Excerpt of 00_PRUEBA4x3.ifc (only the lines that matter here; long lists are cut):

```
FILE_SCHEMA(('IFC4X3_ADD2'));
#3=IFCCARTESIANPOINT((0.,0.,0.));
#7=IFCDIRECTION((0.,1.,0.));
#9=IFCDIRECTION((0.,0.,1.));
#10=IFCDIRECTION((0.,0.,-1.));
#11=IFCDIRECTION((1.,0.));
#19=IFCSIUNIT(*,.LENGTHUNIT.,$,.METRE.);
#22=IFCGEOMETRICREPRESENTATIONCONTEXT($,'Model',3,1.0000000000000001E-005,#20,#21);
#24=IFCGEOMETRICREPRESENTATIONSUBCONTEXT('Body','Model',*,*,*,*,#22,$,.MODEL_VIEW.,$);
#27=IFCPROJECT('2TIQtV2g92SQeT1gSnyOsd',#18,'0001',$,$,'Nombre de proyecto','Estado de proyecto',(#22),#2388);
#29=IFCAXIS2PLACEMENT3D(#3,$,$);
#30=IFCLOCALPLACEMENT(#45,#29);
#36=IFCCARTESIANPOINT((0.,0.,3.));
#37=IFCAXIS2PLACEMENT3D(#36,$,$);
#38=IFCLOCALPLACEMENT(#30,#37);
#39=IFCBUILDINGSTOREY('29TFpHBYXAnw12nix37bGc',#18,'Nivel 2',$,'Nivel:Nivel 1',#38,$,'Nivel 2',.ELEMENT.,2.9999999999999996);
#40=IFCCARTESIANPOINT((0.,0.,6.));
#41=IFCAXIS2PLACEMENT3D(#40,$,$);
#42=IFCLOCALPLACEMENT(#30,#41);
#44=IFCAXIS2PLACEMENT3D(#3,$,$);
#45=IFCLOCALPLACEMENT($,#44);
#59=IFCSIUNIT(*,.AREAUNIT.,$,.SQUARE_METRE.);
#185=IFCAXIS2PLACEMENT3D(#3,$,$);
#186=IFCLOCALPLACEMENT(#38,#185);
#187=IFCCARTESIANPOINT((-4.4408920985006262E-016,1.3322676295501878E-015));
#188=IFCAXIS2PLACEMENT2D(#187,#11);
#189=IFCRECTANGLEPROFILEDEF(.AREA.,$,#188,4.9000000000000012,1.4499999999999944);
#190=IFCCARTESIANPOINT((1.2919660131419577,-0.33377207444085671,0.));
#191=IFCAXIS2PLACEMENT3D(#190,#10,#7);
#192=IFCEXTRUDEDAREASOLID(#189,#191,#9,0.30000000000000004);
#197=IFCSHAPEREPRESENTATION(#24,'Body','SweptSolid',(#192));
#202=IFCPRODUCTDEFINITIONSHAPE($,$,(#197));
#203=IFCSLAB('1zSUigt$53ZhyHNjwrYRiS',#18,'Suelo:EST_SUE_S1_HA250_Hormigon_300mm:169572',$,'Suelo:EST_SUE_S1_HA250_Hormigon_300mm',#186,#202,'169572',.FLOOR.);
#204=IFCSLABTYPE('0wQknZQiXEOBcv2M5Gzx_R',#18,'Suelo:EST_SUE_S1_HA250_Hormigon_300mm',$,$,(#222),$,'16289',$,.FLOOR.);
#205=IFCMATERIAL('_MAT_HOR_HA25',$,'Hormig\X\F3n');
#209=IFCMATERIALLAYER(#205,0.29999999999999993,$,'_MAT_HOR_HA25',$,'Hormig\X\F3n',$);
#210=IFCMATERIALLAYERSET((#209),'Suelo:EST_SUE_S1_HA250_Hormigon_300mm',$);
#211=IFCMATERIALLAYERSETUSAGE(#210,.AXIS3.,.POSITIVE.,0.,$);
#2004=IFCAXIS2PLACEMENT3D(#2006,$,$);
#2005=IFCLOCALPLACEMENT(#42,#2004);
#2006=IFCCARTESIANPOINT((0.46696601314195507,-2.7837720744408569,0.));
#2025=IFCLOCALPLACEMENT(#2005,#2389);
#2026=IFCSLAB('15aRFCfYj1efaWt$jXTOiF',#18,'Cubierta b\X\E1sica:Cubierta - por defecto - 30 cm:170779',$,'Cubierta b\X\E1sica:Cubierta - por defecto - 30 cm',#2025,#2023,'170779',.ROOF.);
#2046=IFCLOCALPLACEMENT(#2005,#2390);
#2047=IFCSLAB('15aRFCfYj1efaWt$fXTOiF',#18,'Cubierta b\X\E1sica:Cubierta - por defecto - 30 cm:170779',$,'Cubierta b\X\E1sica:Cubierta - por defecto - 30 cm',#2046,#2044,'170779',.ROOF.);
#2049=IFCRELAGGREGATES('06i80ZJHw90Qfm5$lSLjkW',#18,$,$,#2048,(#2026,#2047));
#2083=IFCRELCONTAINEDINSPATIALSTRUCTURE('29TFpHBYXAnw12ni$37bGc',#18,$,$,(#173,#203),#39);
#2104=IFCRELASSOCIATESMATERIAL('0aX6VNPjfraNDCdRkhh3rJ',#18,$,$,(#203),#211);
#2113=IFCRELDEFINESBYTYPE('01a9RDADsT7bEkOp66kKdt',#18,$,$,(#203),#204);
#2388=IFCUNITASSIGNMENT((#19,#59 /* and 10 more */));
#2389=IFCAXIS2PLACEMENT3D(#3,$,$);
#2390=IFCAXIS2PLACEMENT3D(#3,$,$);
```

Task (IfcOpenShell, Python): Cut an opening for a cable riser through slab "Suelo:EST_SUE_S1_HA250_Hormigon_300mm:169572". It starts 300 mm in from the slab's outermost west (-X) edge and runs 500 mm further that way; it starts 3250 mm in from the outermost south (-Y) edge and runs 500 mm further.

```python
import numpy as np
import ifcopenshell
import ifcopenshell.api.feature
import ifcopenshell.api.geometry
import ifcopenshell.api.root
import ifcopenshell.geom
import ifcopenshell.util.placement
import ifcopenshell.util.representation
import ifcopenshell.util.shape
import ifcopenshell.util.unit

model = ifcopenshell.open("00_PRUEBA4x3.ifc")
unit_scale = ifcopenshell.util.unit.calculate_unit_scale(model)
settings = ifcopenshell.geom.settings()


def volume(element):
    """Net volume in cubic metres, openings subtracted."""
    shape = ifcopenshell.geom.create_shape(settings, element)
    return ifcopenshell.util.shape.get_volume(shape.geometry)


slab = model.by_guid("1zSUigt$53ZhyHNjwrYRiS")
before = volume(slab)

# Extent in the slab's own axes, in metres. The edges named are its -X and -Y sides.
slab_shape = ifcopenshell.geom.create_shape(settings, slab)
vertices = ifcopenshell.util.shape.get_vertices(slab_shape.geometry)
x_min, y_min, bottom = vertices.min(axis=0)
top = vertices[:, 2].max()

opening = ifcopenshell.api.root.create_entity(model, ifc_class="IfcOpeningElement", name="Cable riser opening", predefined_type="OPENING")
context = ifcopenshell.util.representation.get_context(model, "Model", "Body", "MODEL_VIEW")
width, depth = 0.5, 0.5
outline = [(0.0, 0.0), (width, 0.0), (width, depth), (0.0, depth), (0.0, 0.0)]
# Overshoot both faces by 50 mm so the cut is clean.
shape = ifcopenshell.api.geometry.add_slab_representation(
    model, context=context, depth=top - bottom + 0.1, polyline=outline
)
ifcopenshell.api.geometry.assign_representation(model, product=opening, representation=shape)

matrix = ifcopenshell.util.placement.get_local_placement(slab.ObjectPlacement)
matrix[:, 3] = matrix @ np.append(np.array([x_min + 0.3, y_min + 3.25, bottom - 0.05]) / unit_scale, 1.0)
ifcopenshell.api.geometry.edit_object_placement(model, product=opening, matrix=matrix, is_si=False)
ifcopenshell.api.feature.add_feature(model, feature=opening, element=slab)

after = volume(slab)

print(f"slab volume {before:.3f} -> {after:.3f} m3")

model.write("00_PRUEBA4x3_updated.ifc")
```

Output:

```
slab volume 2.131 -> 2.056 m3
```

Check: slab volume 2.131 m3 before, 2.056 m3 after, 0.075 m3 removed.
